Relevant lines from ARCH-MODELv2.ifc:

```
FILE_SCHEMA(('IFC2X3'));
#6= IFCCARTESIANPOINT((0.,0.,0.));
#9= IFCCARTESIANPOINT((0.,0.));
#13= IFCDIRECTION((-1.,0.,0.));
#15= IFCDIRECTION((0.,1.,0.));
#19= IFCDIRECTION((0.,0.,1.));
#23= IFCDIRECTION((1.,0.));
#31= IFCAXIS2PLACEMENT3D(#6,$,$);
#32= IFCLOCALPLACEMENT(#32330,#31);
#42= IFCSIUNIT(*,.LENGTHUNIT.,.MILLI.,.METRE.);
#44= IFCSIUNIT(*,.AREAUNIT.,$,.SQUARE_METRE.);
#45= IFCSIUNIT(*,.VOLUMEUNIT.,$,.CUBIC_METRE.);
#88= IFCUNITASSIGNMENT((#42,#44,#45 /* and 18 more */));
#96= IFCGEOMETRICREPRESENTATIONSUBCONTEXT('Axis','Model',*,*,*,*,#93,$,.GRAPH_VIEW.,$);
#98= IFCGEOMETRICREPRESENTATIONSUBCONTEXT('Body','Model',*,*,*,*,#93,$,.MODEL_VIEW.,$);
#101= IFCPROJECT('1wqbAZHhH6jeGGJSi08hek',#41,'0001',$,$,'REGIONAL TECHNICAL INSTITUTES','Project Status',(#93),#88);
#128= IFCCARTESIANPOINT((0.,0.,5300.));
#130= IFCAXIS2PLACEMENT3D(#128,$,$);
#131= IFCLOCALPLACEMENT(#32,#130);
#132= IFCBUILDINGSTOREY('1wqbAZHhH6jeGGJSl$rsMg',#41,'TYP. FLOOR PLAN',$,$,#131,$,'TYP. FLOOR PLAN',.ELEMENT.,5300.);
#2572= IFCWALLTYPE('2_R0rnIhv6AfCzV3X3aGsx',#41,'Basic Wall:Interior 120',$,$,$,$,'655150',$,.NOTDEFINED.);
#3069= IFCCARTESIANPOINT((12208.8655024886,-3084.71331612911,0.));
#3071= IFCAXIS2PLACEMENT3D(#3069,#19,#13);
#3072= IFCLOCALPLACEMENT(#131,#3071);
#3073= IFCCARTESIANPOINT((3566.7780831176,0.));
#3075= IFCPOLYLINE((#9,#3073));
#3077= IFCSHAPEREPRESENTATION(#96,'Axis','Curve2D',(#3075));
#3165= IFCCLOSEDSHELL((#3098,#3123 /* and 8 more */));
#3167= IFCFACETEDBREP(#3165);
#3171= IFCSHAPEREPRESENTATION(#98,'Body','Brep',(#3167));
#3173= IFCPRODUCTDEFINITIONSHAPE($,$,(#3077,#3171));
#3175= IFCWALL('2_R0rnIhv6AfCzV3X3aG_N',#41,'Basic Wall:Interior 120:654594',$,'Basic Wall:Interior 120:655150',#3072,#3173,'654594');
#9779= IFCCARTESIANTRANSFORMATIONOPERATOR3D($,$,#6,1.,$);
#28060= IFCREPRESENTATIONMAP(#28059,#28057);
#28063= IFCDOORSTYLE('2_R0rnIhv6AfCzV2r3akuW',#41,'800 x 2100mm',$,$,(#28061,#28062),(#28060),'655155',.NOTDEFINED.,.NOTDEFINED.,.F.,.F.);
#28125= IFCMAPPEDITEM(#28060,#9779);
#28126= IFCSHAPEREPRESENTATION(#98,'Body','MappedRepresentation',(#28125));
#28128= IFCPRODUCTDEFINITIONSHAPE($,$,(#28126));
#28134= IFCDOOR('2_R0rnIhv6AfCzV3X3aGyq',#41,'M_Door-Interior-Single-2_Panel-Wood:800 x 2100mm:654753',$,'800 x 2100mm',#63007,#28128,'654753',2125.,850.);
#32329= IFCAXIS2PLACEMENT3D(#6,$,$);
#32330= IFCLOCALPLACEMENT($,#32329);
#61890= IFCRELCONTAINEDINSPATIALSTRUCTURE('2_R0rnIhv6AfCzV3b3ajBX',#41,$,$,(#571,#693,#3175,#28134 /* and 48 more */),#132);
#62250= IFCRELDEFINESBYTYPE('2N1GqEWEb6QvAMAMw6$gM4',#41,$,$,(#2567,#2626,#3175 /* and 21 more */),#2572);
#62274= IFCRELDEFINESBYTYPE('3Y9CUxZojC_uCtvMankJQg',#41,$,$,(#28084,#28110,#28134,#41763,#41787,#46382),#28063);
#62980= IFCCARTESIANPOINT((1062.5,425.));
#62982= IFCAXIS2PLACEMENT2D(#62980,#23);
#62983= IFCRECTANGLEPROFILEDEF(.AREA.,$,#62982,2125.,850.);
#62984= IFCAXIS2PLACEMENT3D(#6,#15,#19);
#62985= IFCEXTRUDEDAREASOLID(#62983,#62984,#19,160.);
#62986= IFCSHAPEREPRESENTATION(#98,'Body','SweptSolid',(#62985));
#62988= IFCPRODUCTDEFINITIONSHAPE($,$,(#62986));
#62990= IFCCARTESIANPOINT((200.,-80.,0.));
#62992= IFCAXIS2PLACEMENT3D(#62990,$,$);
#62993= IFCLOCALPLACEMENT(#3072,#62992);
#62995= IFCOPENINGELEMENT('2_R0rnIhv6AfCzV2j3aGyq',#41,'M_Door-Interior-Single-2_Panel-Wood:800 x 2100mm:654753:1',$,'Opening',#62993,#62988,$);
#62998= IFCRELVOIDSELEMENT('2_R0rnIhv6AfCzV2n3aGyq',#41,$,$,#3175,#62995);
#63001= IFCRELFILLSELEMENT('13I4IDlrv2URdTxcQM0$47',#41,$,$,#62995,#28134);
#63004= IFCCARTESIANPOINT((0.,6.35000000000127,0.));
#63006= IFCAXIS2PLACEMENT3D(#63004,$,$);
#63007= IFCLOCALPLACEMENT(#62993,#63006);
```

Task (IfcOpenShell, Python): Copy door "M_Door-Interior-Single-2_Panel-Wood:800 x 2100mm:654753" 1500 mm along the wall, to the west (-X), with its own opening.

```python
import ifcopenshell
import ifcopenshell.api.feature
import ifcopenshell.api.geometry
import ifcopenshell.api.root
import ifcopenshell.geom
import ifcopenshell.util.element
import ifcopenshell.util.placement
import ifcopenshell.util.shape
import ifcopenshell.util.unit

model = ifcopenshell.open("ARCH-MODELv2.ifc")
unit_scale = ifcopenshell.util.unit.calculate_unit_scale(model)
settings = ifcopenshell.geom.settings()


def volume(element):
    """Net volume in cubic metres, openings subtracted."""
    shape = ifcopenshell.geom.create_shape(settings, element)
    return ifcopenshell.util.shape.get_volume(shape.geometry)


def reuse_history(source, copy):
    """copy_class also copies each property set's owner history, people and application; keep the originals."""
    for rel in copy.IsDefinedBy:
        if rel.is_a("IfcRelDefinesByProperties") and (history := rel.RelatingPropertyDefinition.OwnerHistory):
            rel.RelatingPropertyDefinition.OwnerHistory = source.OwnerHistory
            ifcopenshell.util.element.remove_deep2(model, history)


door = model.by_guid("2_R0rnIhv6AfCzV3X3aGyq")
opening = door.FillsVoids[0].RelatingOpeningElement
wall = opening.VoidsElements[0].RelatingBuildingElement
before = volume(wall)
shift = ifcopenshell.util.placement.get_local_placement(wall.ObjectPlacement)[:3, 0] * 1.5 / unit_scale

# copy_class copies the void relationship, type, container and properties, but no geometry.
new_opening = ifcopenshell.api.root.copy_class(model, product=opening)
new_opening.Representation = ifcopenshell.util.element.copy_deep(
    model, opening.Representation, exclude=["IfcGeometricRepresentationContext", "IfcRepresentationMap"]
)
new_opening.Name = "M_Door-Interior-Single-2_Panel-Wood:800 x 2100mm"
new_door = ifcopenshell.api.root.copy_class(model, product=door)
new_door.Representation = ifcopenshell.util.element.copy_deep(
    model, door.Representation, exclude=["IfcGeometricRepresentationContext", "IfcRepresentationMap"]
)
new_door.Name = "M_Door-Interior-Single-2_Panel-Wood:800 x 2100mm"
new_door.Tag = None
reuse_history(door, new_door)
fills = ifcopenshell.api.feature.add_filling(model, opening=new_opening, element=new_door)
fills.OwnerHistory = new_door.OwnerHistory  # required in IFC2X3

for old, new in ((opening, new_opening), (door, new_door)):
    matrix = ifcopenshell.util.placement.get_local_placement(old.ObjectPlacement)
    matrix[:3, 3] += shift
    ifcopenshell.api.geometry.edit_object_placement(model, product=new, matrix=matrix, is_si=False)

after = volume(wall)

print(f"wall volume {before:.3f} -> {after:.3f} m3")

model.write("ARCH-MODELv2-out.ifc")
```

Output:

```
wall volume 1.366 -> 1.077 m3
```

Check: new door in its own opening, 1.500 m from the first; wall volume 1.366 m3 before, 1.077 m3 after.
